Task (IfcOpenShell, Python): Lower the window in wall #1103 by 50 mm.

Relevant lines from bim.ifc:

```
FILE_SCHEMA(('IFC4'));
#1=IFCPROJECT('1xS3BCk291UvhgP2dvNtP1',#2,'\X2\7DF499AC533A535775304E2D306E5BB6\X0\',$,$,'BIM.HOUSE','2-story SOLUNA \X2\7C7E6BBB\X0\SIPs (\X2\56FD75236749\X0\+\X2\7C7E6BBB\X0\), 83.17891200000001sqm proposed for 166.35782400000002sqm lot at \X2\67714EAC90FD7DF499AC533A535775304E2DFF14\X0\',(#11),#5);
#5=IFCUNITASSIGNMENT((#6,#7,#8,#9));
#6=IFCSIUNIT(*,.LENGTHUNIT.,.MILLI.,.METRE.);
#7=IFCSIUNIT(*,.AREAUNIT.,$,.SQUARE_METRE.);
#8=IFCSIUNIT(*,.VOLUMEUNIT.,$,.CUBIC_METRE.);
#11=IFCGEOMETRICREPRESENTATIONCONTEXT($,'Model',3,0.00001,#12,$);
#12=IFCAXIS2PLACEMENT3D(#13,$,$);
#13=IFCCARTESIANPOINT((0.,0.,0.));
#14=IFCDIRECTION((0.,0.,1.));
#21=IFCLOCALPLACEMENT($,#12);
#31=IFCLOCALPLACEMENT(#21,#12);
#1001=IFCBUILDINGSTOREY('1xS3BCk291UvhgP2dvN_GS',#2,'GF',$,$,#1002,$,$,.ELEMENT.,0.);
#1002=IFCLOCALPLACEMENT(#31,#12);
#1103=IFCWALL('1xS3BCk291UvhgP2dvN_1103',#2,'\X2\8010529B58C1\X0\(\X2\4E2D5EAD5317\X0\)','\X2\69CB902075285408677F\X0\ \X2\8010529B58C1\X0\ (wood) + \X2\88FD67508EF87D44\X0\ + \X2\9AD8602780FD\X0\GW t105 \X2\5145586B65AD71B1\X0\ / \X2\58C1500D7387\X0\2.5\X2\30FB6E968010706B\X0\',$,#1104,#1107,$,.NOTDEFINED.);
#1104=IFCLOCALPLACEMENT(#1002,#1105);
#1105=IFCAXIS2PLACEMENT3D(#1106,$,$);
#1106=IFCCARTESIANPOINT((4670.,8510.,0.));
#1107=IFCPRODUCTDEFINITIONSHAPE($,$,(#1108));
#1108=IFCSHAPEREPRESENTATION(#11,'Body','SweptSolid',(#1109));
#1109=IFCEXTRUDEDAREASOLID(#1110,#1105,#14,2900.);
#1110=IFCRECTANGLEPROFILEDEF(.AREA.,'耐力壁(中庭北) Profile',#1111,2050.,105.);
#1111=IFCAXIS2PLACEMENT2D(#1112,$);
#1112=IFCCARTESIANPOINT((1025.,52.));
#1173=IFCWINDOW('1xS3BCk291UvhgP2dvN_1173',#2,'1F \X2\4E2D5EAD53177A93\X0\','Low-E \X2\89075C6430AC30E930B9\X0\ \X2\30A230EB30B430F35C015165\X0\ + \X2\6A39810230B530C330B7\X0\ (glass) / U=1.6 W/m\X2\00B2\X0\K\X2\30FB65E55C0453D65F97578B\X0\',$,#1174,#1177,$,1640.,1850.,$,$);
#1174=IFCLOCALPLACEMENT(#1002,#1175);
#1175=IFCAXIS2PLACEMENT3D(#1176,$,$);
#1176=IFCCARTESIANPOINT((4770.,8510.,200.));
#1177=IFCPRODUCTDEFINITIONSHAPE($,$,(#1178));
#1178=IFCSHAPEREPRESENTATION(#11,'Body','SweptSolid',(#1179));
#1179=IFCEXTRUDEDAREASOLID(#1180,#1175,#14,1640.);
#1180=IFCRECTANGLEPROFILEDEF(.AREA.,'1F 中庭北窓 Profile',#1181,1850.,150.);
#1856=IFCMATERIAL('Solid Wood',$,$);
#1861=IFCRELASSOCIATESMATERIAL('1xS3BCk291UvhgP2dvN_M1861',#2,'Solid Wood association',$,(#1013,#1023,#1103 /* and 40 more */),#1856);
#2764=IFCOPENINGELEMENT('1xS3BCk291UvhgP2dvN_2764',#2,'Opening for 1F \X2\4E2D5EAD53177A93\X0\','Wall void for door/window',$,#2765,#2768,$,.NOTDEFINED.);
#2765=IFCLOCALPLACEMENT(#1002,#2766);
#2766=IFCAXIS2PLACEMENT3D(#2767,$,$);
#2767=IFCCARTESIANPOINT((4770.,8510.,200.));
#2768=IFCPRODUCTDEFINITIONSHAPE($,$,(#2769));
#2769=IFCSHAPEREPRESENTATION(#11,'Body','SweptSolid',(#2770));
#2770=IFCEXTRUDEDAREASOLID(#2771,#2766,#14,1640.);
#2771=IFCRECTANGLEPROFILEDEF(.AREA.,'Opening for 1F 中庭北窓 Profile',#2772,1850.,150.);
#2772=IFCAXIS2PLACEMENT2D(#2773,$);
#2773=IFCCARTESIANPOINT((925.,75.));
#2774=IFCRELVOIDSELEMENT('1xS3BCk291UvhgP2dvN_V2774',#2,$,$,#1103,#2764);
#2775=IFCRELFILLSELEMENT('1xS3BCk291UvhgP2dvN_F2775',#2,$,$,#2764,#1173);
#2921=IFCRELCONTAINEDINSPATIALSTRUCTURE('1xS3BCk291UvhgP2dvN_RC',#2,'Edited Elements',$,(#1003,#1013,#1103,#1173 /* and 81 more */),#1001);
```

```python
import numpy as np
import ifcopenshell
import ifcopenshell.api.geometry
import ifcopenshell.util.placement
import ifcopenshell.util.unit

model = ifcopenshell.open("bim.ifc")
unit_scale = ifcopenshell.util.unit.calculate_unit_scale(model)

window = model.by_guid("1xS3BCk291UvhgP2dvN_1173")
opening = window.FillsVoids[0].RelatingOpeningElement
dz = -0.05 / unit_scale

shift = np.array([0.0, 0.0, dz])
# The window is not placed relative to its opening, so move both.
for product in (opening, window):
    matrix = ifcopenshell.util.placement.get_local_placement(product.ObjectPlacement)
    matrix[:3, 3] += shift
    ifcopenshell.api.geometry.edit_object_placement(model, product=product, matrix=matrix, is_si=False)

print(f"moved by {dz * unit_scale:+.3f} m")

model.write("bim_updated.ifc")
```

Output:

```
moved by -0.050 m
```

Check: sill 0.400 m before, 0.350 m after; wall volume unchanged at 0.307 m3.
